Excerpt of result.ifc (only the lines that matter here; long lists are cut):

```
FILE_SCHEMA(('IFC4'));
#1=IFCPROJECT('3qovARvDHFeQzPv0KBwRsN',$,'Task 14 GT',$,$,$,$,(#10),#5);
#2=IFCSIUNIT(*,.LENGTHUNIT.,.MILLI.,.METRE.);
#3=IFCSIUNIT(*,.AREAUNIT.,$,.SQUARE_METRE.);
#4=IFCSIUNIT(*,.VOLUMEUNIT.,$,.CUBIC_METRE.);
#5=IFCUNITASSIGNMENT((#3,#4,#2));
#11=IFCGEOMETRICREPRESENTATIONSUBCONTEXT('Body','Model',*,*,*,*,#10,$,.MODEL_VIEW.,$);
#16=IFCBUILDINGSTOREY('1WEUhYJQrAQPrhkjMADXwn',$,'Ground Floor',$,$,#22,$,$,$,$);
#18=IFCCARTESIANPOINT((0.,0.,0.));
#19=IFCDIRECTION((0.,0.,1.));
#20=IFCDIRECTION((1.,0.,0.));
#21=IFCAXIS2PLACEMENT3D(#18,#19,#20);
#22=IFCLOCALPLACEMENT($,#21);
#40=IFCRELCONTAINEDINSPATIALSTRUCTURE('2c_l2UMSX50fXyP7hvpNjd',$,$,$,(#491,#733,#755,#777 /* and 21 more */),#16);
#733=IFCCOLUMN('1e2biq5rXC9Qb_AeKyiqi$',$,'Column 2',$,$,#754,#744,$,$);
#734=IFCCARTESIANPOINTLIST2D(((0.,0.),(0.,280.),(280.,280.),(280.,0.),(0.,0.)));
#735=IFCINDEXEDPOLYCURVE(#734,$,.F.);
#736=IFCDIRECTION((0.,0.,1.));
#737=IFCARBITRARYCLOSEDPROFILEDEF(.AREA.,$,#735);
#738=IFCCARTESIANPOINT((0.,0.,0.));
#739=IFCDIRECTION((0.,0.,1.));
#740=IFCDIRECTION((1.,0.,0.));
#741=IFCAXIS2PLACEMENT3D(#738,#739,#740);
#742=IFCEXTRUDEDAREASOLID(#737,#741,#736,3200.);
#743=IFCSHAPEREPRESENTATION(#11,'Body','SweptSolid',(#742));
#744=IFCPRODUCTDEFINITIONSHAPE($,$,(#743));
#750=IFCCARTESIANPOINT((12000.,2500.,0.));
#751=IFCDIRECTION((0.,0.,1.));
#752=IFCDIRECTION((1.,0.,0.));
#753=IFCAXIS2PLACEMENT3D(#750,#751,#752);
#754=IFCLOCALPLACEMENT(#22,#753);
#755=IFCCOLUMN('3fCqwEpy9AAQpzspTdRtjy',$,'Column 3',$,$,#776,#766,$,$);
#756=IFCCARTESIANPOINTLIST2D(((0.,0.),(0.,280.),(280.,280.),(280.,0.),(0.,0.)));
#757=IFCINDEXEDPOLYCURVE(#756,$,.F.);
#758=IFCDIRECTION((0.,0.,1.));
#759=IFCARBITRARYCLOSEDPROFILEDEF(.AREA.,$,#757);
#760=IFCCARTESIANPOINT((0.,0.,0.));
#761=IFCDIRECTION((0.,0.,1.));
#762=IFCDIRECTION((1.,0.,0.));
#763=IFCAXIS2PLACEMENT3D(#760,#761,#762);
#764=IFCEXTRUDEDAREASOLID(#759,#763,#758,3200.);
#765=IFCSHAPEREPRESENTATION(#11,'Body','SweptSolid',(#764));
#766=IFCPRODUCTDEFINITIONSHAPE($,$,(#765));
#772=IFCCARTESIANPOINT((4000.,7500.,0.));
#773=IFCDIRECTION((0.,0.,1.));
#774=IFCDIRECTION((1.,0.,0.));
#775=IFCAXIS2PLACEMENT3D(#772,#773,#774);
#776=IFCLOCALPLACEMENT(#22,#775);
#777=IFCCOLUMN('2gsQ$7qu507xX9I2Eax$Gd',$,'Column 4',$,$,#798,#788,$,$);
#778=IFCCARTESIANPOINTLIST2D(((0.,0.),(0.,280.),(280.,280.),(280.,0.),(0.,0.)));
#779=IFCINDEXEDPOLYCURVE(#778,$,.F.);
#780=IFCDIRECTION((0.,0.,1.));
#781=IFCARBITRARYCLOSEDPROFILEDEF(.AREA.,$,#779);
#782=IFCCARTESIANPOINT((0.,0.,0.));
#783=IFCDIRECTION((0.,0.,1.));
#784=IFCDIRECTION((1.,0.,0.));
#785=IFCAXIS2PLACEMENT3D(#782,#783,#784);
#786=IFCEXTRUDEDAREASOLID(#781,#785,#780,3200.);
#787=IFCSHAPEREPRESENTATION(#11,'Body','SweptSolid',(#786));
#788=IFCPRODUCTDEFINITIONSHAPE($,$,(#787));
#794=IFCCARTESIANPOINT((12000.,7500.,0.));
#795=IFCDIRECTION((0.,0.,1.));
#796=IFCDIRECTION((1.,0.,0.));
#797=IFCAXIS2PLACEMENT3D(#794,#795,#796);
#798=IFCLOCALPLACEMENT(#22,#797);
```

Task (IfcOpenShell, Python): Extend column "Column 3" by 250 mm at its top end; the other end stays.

```python
import ifcopenshell
import ifcopenshell.util.representation
import ifcopenshell.util.unit

model = ifcopenshell.open("result.ifc")
unit_scale = ifcopenshell.util.unit.calculate_unit_scale(model)

member = model.by_guid("3fCqwEpy9AAQpzspTdRtjy")
change = 0.25 / unit_scale

# The extrusion runs towards the end named, so only its depth changes.
body = ifcopenshell.util.representation.get_representation(member, "Model", "Body")
solid = body.Items[0]
old_length = solid.Depth
solid.Depth += change

print(f"length {old_length:g} -> {solid.Depth:g}")

model.write("result-out.ifc")
```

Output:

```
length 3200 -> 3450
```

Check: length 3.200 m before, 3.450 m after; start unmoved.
